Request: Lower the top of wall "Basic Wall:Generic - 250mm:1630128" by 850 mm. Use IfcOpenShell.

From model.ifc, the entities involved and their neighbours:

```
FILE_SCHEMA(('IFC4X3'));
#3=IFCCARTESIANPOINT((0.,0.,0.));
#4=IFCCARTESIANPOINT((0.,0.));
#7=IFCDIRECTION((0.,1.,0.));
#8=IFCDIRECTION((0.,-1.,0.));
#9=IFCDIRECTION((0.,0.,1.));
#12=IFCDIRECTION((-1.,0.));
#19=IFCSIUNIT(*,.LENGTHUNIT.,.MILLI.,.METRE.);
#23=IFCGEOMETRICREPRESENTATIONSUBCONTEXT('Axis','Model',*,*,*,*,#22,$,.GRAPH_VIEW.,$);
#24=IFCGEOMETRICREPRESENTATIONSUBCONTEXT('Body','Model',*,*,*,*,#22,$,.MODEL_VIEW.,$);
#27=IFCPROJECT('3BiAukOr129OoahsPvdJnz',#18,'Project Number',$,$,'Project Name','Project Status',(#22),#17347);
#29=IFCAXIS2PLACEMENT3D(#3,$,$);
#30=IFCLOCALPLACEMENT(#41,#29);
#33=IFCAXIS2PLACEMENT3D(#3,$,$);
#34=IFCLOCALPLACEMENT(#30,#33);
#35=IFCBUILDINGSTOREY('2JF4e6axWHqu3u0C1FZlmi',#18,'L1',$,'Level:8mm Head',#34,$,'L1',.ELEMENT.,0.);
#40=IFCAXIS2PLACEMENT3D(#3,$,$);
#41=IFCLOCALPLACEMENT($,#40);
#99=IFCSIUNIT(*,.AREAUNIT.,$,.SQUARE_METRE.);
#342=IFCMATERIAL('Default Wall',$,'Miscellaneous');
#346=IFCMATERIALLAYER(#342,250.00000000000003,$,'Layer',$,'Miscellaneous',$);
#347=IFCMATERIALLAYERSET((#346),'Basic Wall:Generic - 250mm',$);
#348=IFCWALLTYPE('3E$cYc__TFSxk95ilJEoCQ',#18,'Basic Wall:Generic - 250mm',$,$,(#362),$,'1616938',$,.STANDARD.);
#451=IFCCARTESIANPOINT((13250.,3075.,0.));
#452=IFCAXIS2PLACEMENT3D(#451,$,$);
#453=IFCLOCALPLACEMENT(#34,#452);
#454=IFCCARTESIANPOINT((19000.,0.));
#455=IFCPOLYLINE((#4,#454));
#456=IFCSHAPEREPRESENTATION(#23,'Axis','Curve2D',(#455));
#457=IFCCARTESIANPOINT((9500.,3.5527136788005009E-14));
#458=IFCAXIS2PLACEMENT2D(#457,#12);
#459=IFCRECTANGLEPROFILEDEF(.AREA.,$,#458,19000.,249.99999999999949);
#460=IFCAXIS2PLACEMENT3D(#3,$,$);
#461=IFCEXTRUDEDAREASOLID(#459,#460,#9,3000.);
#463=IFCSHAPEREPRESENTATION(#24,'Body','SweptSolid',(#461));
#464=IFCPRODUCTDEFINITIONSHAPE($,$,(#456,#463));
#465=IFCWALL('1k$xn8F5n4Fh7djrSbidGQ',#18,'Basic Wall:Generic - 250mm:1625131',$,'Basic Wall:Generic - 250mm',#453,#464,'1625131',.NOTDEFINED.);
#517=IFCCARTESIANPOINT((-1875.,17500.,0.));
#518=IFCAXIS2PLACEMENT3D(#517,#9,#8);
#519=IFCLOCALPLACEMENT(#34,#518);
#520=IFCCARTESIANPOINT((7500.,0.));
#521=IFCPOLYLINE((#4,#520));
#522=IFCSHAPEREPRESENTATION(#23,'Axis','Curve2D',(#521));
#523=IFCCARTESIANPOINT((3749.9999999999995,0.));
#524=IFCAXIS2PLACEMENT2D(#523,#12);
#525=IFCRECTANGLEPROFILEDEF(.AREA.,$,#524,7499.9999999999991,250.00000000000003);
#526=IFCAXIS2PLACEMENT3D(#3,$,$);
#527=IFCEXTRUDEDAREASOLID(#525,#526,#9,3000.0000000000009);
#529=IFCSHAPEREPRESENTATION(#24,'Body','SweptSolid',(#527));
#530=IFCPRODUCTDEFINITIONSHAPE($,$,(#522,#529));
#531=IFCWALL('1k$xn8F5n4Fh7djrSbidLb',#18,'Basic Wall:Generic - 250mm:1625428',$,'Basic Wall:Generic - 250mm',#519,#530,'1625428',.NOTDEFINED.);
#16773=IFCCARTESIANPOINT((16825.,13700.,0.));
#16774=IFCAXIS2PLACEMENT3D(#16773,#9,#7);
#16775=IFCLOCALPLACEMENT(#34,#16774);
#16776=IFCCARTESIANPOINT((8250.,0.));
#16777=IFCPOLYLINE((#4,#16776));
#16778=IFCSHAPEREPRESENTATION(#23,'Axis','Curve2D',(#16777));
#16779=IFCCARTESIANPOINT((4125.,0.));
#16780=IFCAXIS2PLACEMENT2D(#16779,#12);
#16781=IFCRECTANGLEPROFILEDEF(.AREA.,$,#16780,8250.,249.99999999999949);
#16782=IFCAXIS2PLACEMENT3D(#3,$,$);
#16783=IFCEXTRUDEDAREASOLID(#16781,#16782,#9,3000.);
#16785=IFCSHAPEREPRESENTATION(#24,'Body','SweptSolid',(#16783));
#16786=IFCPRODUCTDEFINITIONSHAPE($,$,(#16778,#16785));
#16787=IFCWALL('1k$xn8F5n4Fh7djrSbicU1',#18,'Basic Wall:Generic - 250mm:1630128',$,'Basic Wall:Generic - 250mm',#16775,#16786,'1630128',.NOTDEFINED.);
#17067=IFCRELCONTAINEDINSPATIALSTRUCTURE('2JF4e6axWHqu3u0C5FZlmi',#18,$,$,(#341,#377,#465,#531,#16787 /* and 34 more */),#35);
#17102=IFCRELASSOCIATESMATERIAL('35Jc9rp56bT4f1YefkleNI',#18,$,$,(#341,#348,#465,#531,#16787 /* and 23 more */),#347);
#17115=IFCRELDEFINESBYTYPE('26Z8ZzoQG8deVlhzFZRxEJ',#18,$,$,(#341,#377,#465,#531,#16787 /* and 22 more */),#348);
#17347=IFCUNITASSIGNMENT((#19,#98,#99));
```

```python
import ifcopenshell
import ifcopenshell.geom
import ifcopenshell.util.representation
import ifcopenshell.util.shape
import ifcopenshell.util.unit

model = ifcopenshell.open("model.ifc")
unit_scale = ifcopenshell.util.unit.calculate_unit_scale(model)
settings = ifcopenshell.geom.settings()


def volume(element):
    """Net volume in cubic metres, openings subtracted."""
    shape = ifcopenshell.geom.create_shape(settings, element)
    return ifcopenshell.util.shape.get_volume(shape.geometry)


wall = model.by_guid("1k$xn8F5n4Fh7djrSbicU1")
before = volume(wall)

body = ifcopenshell.util.representation.get_representation(wall, "Model", "Body")
solid = body.Items[0]
old_height = solid.Depth
solid.Depth -= 0.85 / unit_scale
after = volume(wall)

print(f"height {old_height:g} -> {solid.Depth:g}, volume {before:.3f} -> {after:.3f} m3")

model.write("model_edited.ifc")
```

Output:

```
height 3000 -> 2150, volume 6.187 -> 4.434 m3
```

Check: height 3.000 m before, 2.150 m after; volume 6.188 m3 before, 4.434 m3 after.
